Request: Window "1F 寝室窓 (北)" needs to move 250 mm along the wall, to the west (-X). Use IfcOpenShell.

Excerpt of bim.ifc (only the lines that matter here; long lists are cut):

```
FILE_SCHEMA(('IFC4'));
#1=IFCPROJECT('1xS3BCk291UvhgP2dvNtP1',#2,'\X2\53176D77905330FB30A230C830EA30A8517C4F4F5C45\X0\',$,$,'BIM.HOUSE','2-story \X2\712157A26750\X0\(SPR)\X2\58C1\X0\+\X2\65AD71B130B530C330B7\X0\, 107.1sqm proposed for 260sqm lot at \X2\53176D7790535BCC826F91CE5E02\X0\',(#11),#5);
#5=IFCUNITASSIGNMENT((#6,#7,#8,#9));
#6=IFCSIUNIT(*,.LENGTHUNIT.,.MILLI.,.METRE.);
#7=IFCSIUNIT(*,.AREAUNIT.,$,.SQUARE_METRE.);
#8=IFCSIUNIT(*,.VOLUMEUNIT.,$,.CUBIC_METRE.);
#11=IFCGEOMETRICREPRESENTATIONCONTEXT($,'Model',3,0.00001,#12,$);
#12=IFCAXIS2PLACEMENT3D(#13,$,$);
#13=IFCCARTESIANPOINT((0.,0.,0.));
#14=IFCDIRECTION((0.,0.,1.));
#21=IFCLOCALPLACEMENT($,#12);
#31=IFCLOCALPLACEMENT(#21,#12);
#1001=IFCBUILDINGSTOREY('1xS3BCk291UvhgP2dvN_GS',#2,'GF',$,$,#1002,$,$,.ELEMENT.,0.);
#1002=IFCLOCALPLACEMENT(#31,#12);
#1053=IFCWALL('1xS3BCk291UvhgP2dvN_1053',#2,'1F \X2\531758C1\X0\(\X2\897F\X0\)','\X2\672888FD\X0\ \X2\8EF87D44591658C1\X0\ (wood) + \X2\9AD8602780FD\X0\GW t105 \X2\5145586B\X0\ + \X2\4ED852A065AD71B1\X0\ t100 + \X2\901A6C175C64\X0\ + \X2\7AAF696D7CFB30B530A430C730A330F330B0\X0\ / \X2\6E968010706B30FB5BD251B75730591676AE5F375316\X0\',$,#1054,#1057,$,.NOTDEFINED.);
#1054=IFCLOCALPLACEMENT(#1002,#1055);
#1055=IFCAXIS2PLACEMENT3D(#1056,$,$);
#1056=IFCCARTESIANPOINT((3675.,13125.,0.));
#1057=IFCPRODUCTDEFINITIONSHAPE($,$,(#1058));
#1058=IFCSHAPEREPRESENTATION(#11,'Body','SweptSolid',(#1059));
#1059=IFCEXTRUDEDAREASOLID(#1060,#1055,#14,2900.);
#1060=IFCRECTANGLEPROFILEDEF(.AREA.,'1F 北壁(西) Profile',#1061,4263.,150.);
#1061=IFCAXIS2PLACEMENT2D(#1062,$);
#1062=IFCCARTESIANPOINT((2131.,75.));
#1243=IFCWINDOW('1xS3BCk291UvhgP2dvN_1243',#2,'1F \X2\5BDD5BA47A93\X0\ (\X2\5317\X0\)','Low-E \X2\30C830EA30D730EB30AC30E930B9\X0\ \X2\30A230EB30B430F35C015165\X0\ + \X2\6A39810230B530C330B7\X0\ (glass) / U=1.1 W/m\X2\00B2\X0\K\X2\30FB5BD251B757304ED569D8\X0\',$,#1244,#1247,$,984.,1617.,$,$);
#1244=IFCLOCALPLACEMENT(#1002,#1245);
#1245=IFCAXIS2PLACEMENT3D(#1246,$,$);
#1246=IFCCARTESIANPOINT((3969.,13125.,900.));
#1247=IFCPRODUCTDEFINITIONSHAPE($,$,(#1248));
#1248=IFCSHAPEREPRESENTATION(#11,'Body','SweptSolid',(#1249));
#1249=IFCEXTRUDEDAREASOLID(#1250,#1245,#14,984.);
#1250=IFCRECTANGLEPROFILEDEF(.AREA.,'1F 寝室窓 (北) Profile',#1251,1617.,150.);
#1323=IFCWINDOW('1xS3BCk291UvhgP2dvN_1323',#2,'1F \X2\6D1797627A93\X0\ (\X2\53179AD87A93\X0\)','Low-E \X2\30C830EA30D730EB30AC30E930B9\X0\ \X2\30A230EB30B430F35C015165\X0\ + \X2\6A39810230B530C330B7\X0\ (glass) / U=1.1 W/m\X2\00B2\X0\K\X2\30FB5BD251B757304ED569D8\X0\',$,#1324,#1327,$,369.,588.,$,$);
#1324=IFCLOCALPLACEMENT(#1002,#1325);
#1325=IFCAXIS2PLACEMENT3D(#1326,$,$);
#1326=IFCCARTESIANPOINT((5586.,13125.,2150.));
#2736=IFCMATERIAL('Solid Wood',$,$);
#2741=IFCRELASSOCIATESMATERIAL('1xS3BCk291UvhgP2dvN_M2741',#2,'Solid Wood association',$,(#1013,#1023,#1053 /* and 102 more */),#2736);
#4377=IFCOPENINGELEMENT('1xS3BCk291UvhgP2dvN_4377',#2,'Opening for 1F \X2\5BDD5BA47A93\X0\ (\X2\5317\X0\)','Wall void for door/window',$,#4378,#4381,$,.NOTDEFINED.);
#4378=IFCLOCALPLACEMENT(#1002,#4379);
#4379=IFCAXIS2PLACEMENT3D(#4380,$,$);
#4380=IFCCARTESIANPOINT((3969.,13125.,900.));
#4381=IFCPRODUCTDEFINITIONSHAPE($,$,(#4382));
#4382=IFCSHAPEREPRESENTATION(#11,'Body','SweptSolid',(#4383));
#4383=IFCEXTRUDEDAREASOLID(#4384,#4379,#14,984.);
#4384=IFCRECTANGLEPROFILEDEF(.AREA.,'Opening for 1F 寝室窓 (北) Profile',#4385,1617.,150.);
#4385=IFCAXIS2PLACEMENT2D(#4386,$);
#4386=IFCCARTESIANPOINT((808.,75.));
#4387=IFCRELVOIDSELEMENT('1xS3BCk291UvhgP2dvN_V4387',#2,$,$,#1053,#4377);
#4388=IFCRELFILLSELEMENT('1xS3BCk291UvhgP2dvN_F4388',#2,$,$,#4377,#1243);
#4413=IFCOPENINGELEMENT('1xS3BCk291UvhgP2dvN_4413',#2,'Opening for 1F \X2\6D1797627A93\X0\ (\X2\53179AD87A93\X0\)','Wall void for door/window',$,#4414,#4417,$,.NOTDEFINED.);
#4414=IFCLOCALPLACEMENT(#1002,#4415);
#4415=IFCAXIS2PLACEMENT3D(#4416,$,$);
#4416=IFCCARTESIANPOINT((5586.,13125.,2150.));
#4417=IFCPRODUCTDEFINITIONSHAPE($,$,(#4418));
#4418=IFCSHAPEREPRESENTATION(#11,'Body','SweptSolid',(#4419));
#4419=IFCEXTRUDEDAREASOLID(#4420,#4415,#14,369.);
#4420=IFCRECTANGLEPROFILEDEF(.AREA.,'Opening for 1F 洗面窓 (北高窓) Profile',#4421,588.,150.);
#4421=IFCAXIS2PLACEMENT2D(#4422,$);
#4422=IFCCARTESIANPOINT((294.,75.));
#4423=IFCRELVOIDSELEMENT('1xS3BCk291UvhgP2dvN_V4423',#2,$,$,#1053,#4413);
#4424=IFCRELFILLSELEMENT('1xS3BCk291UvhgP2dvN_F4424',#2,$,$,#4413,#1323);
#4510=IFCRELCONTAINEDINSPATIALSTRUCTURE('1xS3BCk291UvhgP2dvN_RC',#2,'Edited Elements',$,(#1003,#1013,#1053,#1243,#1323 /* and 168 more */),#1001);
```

```python
import ifcopenshell
import ifcopenshell.api.geometry
import ifcopenshell.util.placement

model = ifcopenshell.open("bim.ifc")

window = model.by_id(1243)
opening = window.FillsVoids[0].RelatingOpeningElement
wall = opening.VoidsElements[0].RelatingBuildingElement

wall_matrix = ifcopenshell.util.placement.get_local_placement(wall.ObjectPlacement)
shift = wall_matrix[:3, 0] * -250.0
before = ifcopenshell.util.placement.get_local_placement(window.ObjectPlacement)[:3, 3].copy()

# The window is not placed relative to its opening, so move both.
for product in (opening, window):
    matrix = ifcopenshell.util.placement.get_local_placement(product.ObjectPlacement)
    matrix[:3, 3] += shift
    ifcopenshell.api.geometry.edit_object_placement(model, product=product, matrix=matrix, is_si=False)

after = ifcopenshell.util.placement.get_local_placement(window.ObjectPlacement)[:3, 3]
print("window moved by", (after - before).round(3) + 0.0)

model.write("bim_edited.ifc")
```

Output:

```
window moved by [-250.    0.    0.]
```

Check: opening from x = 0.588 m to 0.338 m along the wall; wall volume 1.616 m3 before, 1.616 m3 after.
